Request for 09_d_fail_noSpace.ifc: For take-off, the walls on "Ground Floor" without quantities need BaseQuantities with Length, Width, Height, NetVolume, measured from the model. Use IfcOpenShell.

First a look at what the model holds.

```python
import ifcopenshell
import ifcopenshell.util.element
import ifcopenshell.util.unit

model = ifcopenshell.open("09_d_fail_noSpace.ifc")
print(model.schema)
for unit_type in ("LENGTHUNIT", "AREAUNIT", "VOLUMEUNIT"):
    print(unit_type, ifcopenshell.util.unit.calculate_unit_scale(model, unit_type))
storey = next(s for s in model.by_type("IfcBuildingStorey") if s.Name == "Ground Floor")
walls = [e for e in ifcopenshell.util.element.get_decomposition(storey) if e.is_a("IfcWall")]
for e in sorted(walls, key=lambda e: e.id()):
    print(e.id(), e.is_a(), e.Name, list(ifcopenshell.util.element.get_psets(e, qtos_only=True)), sep=" | ")
```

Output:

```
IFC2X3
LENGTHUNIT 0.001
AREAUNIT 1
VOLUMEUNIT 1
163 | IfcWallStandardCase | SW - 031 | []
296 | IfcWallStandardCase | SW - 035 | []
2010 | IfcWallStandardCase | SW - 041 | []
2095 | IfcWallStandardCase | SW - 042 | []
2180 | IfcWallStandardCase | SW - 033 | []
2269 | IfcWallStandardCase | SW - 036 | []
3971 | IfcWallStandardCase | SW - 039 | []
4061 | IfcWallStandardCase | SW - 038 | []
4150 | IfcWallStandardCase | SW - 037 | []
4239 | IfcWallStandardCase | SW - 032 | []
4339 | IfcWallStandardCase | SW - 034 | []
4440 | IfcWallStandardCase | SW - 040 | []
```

```python
import ifcopenshell
import ifcopenshell.api.pset
import ifcopenshell.geom
import ifcopenshell.util.element
import ifcopenshell.util.shape
import ifcopenshell.util.unit

model = ifcopenshell.open("09_d_fail_noSpace.ifc")
unit_scale = ifcopenshell.util.unit.calculate_unit_scale(model)
volume_scale = ifcopenshell.util.unit.calculate_unit_scale(model, "VOLUMEUNIT")
settings = ifcopenshell.geom.settings()

storey = next(s for s in model.by_type("IfcBuildingStorey") if s.Name == "Ground Floor")
walls = [e for e in ifcopenshell.util.element.get_decomposition(storey) if e.is_a("IfcWall")]

for e in sorted(walls, key=lambda e: e.id()):
    if ifcopenshell.util.element.get_psets(e, qtos_only=True, should_inherit=False):
        continue
    # Geometry comes back in metres, in the element's own axes.
    shape = ifcopenshell.geom.create_shape(settings, e)
    values = {
        "Length": ifcopenshell.util.shape.get_x(shape.geometry) / unit_scale,
        "Width": ifcopenshell.util.shape.get_y(shape.geometry) / unit_scale,
        "Height": ifcopenshell.util.shape.get_z(shape.geometry) / unit_scale,
        "NetVolume": ifcopenshell.util.shape.get_volume(shape.geometry) / volume_scale,
    }
    qto = ifcopenshell.api.pset.add_qto(model, product=e, name="BaseQuantities")
    ifcopenshell.api.pset.edit_qto(model, qto=qto, properties=values)
    print(e.id(), {k: round(v, 3) for k, v in values.items()})

model.write("09_d_fail_noSpace-out.ifc")
```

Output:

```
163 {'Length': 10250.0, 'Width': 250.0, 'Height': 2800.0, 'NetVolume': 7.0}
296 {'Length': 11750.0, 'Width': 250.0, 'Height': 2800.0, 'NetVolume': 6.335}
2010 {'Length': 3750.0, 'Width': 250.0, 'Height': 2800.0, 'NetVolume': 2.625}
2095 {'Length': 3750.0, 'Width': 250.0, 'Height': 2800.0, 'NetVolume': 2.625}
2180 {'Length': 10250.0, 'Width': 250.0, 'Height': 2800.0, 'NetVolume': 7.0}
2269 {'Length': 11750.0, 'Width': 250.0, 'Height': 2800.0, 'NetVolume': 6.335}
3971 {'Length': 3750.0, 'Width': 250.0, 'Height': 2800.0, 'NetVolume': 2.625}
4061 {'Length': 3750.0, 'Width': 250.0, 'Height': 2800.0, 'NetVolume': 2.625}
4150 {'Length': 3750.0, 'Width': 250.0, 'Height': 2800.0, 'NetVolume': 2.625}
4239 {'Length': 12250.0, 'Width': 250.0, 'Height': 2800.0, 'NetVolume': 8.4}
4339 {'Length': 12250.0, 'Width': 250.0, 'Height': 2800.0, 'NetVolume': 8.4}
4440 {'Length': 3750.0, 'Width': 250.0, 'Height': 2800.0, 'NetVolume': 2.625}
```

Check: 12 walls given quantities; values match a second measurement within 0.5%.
